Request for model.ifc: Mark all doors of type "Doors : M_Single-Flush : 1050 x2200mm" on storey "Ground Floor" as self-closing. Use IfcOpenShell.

First a look at what the model holds.

```python
import ifcopenshell
import ifcopenshell.util.element

model = ifcopenshell.open("model.ifc")
print(model.schema)
storey = next(s for s in model.by_type("IfcBuildingStorey") if s.Name == "Ground Floor")
doors = [e for e in ifcopenshell.util.element.get_decomposition(storey) if e.is_a("IfcDoor")]
seen = {}
for e in doors:
    element_type = ifcopenshell.util.element.get_type(e)
    key = (element_type.Name if element_type != e and element_type else None, ifcopenshell.util.element.get_pset(e, "Pset_DoorCommon", "SelfClosing"))
    seen[key] = seen.get(key, 0) + 1
for (name, value), count in sorted(seen.items(), key=str):
    print(count, "x", name, "|", value)
```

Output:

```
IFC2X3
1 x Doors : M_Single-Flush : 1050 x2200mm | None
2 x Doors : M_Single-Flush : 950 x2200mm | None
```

```python
import ifcopenshell
import ifcopenshell.api.pset
import ifcopenshell.util.element

model = ifcopenshell.open("model.ifc")

storey = next(s for s in model.by_type("IfcBuildingStorey") if s.Name == "Ground Floor")
doors = [e for e in ifcopenshell.util.element.get_decomposition(storey) if e.is_a("IfcDoor")]

count = 0
for e in doors:
    element_type = ifcopenshell.util.element.get_type(e)
    if element_type in (None, e) or element_type.Name != "Doors : M_Single-Flush : 1050 x2200mm":
        continue
    # add_pset returns the element's existing set when there is one.
    pset = ifcopenshell.api.pset.add_pset(model, product=e, name="Pset_DoorCommon")
    ifcopenshell.api.pset.edit_pset(model, pset=pset, properties={"SelfClosing": True})
    count += 1

print(count, "doors updated")

model.write("model_rev.ifc")
```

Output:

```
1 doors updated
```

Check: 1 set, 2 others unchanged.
